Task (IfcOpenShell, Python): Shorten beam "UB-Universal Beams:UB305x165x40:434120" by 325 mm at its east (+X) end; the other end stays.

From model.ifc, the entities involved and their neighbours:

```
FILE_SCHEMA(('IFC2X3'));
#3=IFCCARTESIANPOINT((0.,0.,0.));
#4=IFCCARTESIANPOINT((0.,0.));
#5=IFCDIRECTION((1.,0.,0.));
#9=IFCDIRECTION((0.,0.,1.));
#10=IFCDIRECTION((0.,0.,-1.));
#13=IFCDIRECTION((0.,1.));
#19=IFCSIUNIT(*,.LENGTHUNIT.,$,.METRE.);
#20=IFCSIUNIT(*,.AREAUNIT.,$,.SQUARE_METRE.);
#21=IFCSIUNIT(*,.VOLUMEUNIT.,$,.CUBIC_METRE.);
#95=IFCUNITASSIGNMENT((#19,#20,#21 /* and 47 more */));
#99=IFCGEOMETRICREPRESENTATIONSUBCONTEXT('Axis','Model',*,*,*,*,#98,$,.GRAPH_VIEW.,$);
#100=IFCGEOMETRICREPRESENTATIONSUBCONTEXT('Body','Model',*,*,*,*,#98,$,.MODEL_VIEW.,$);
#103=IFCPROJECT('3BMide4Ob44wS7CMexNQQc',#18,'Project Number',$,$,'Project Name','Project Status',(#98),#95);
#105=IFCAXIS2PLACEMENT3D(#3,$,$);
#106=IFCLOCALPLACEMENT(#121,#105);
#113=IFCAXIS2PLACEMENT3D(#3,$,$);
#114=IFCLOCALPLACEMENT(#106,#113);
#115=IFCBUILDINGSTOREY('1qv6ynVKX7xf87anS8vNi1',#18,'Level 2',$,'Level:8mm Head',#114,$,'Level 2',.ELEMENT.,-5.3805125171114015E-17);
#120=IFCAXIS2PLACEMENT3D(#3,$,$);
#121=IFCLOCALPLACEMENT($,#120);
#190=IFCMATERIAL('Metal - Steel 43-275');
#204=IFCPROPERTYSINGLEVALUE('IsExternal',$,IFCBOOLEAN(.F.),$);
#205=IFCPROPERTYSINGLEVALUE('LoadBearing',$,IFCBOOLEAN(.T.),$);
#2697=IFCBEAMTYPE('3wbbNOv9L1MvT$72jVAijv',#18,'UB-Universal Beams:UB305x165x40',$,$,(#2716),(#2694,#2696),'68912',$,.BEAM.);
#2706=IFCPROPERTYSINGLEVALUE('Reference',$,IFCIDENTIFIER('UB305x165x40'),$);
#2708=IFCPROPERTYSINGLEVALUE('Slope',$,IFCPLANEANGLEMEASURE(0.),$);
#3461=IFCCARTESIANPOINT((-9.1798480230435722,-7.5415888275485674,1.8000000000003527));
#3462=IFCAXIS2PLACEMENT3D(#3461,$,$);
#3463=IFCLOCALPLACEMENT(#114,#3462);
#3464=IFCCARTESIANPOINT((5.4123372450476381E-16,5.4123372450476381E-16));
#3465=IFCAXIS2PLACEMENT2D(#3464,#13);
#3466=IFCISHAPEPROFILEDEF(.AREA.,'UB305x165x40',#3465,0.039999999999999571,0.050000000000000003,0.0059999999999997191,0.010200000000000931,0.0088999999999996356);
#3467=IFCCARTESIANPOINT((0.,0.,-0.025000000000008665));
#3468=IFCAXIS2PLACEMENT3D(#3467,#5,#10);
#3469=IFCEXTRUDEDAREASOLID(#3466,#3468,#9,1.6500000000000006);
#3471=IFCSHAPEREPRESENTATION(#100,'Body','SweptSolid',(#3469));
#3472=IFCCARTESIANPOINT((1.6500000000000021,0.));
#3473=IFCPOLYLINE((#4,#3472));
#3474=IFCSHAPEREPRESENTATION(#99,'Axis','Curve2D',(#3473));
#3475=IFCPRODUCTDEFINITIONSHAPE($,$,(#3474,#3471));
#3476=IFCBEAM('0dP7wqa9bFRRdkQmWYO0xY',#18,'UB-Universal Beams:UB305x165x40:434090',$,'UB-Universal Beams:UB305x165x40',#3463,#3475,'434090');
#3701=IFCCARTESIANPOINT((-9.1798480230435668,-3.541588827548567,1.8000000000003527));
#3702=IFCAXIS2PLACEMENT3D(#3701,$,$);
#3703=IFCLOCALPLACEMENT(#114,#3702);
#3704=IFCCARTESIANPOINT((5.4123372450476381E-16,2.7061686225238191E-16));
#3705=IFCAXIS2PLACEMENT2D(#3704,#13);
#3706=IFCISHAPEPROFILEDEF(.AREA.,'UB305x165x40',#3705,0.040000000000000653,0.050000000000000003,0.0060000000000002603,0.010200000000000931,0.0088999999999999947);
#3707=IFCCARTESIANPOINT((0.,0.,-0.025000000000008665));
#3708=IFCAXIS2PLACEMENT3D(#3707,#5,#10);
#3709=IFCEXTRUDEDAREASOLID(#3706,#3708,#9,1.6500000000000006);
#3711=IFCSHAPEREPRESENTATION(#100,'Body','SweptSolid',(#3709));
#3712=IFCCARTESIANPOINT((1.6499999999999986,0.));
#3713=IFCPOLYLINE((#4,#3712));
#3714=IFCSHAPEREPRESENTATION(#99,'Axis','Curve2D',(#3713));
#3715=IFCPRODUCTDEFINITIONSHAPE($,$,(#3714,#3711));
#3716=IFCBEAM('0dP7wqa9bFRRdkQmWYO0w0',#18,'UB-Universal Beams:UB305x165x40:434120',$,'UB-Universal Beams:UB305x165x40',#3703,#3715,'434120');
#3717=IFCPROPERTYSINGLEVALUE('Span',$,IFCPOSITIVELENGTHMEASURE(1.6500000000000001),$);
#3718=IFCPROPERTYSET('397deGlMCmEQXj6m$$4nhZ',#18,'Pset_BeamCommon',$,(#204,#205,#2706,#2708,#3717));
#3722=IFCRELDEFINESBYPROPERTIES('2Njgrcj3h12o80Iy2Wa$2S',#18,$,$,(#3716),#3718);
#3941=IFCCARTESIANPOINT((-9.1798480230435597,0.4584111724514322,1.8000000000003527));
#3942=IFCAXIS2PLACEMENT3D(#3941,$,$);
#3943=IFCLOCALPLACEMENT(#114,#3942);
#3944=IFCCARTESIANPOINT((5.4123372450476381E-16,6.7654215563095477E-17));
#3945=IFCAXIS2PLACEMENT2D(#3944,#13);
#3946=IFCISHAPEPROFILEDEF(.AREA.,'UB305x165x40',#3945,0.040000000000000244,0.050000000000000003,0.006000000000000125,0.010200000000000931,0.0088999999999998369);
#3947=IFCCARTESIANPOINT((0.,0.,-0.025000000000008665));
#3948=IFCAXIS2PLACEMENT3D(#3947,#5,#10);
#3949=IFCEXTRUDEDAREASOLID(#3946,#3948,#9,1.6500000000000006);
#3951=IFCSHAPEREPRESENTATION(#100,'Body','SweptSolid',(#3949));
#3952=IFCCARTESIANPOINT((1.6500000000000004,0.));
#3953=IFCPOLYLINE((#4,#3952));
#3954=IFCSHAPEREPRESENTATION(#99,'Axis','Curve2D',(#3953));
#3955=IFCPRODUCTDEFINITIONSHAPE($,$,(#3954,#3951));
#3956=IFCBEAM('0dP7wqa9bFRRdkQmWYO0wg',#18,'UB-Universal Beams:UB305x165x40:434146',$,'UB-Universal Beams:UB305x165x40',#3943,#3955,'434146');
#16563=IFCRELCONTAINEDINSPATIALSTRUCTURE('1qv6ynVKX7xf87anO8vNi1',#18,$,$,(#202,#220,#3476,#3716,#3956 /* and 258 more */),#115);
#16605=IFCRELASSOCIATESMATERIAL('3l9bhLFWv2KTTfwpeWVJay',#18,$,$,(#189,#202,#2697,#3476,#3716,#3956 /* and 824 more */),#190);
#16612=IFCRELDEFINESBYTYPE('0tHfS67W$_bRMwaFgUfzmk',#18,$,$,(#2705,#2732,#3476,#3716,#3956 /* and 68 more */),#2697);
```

```python
import numpy as np
import ifcopenshell
import ifcopenshell.api.pset
import ifcopenshell.util.element
import ifcopenshell.util.representation
import ifcopenshell.util.unit

model = ifcopenshell.open("model.ifc")
unit_scale = ifcopenshell.util.unit.calculate_unit_scale(model)

member = model.by_id(3716)
change = -0.325 / unit_scale

# The extrusion runs towards the end named, so only its depth changes.
body = ifcopenshell.util.representation.get_representation(member, "Model", "Body")
solid = body.Items[0]
old_length = solid.Depth
solid.Depth += change

# Move the axis end point with it.
axis = next(r for r in member.Representation.Representations if r.RepresentationIdentifier == "Axis").Items[0]
start, end = (np.array(p.Coordinates) for p in axis.Points)
end = end + (end - start) / np.linalg.norm(end - start) * change
point = model.createIfcCartesianPoint(end.tolist())
axis.Points = [axis.Points[0], point]

# Update the stored length and volume.
pset = model.by_id(ifcopenshell.util.element.get_pset(member, "Pset_BeamCommon", should_inherit=False)["id"])
ifcopenshell.api.pset.edit_pset(model, pset=pset, properties={
    "Span": model.create_entity("IfcPositiveLengthMeasure", solid.Depth),
})

print(f"length {old_length:g} -> {solid.Depth:g}")

model.write("model-out.ifc")
```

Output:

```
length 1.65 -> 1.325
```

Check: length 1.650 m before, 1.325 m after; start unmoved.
